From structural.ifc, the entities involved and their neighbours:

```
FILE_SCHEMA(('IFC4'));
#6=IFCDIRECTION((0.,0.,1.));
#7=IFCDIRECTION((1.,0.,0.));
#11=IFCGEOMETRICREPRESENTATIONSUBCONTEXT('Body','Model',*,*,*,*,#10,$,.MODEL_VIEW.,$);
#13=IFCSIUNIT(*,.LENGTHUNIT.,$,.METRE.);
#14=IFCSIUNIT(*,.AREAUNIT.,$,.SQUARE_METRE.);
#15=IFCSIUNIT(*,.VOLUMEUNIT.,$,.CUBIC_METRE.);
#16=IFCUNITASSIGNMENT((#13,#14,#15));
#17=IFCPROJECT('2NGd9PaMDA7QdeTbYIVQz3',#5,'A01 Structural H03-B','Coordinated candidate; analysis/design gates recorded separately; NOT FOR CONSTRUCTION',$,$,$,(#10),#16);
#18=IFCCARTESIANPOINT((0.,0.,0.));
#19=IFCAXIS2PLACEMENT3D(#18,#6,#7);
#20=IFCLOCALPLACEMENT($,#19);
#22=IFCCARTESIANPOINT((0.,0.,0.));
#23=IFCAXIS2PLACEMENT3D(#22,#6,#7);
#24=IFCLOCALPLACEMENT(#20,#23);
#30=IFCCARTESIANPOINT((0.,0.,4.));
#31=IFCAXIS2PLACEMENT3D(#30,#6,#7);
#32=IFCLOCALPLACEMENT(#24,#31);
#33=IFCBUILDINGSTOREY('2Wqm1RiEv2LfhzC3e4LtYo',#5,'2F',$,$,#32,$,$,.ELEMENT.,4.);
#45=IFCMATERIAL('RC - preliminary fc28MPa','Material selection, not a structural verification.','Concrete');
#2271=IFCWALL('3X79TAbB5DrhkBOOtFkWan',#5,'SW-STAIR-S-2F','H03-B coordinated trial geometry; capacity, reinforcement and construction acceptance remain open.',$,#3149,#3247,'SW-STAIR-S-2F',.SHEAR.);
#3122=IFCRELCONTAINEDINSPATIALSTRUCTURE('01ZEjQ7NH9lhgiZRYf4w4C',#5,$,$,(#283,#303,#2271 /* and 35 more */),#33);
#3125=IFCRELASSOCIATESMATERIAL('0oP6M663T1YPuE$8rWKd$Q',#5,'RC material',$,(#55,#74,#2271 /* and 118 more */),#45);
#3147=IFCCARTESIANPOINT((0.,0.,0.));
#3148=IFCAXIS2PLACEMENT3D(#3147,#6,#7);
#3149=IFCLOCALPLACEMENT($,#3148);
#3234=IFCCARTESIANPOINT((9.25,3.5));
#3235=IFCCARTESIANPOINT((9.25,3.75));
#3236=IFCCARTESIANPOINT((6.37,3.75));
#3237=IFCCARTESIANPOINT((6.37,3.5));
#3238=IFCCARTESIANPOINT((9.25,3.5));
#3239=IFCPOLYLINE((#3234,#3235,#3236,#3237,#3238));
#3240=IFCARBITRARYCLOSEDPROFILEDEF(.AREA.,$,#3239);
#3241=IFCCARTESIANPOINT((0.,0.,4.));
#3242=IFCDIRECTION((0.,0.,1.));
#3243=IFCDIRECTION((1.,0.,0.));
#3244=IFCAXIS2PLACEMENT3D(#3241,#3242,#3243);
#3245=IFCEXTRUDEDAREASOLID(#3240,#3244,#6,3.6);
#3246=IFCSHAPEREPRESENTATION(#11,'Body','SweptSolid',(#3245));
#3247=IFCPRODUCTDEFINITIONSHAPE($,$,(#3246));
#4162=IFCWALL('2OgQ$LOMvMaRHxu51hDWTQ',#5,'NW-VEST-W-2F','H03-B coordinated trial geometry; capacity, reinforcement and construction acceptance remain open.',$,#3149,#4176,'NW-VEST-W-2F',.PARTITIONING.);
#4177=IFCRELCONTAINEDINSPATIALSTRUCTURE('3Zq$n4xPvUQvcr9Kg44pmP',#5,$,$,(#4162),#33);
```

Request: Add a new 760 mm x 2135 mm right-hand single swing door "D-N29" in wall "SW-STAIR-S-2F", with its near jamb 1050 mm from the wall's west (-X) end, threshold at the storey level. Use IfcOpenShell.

```python
import numpy as np
import ifcopenshell
import ifcopenshell.api.feature
import ifcopenshell.api.geometry
import ifcopenshell.api.root
import ifcopenshell.api.spatial
import ifcopenshell.geom
import ifcopenshell.util.element
import ifcopenshell.util.placement
import ifcopenshell.util.representation
import ifcopenshell.util.shape
import ifcopenshell.util.unit

model = ifcopenshell.open("structural.ifc")
unit_scale = ifcopenshell.util.unit.calculate_unit_scale(model)
settings = ifcopenshell.geom.settings()


def volume(element):
    """Net volume in cubic metres, openings subtracted."""
    shape = ifcopenshell.geom.create_shape(settings, element)
    return ifcopenshell.util.shape.get_volume(shape.geometry)


wall = model.by_guid("3X79TAbB5DrhkBOOtFkWan")
storey = ifcopenshell.util.element.get_container(wall, ifc_class="IfcBuildingStorey")
context = ifcopenshell.util.representation.get_context(model, "Model", "Body", "MODEL_VIEW")
before = volume(wall)

width, height, from_end, sill = 0.76, 2.135, 1.05, 0.0  # metres

# The wall runs along its own X axis, and the end named is its -X end.
wall_shape = ifcopenshell.geom.create_shape(settings, wall)
x, y, z = ifcopenshell.util.shape.get_vertices(wall_shape.geometry).T
start = x.min() + from_end
face, thickness = float(y.min()), float(y.max() - y.min())
wall_matrix = ifcopenshell.util.placement.get_local_placement(wall.ObjectPlacement)
level = ifcopenshell.util.placement.get_local_placement(storey.ObjectPlacement)[2, 3]


def in_wall(x, y):
    """Placement at x, y metres in the wall's axes, at sill height."""
    matrix = wall_matrix.copy()
    matrix[:, 3] = wall_matrix @ np.array([x / unit_scale, y / unit_scale, 0.0, 1.0])
    matrix[2, 3] = level + sill / unit_scale
    return matrix


# Opening: a box that overshoots both wall faces by 50 mm.
opening = ifcopenshell.api.root.create_entity(model, ifc_class="IfcOpeningElement", predefined_type="OPENING")
box = ifcopenshell.api.geometry.add_wall_representation(
    model, context=context, length=width, height=height, thickness=thickness + 0.1
)
ifcopenshell.api.geometry.assign_representation(model, product=opening, representation=box)
ifcopenshell.api.geometry.edit_object_placement(model, product=opening, matrix=in_wall(start, face - 0.05), is_si=False)
ifcopenshell.api.feature.add_feature(model, feature=opening, element=wall)

door = ifcopenshell.api.root.create_entity(model, ifc_class="IfcDoor", name="D-N29", predefined_type="DOOR")
door.OverallWidth, door.OverallHeight = width / unit_scale, height / unit_scale
door.OperationType = "SINGLE_SWING_RIGHT"
body = ifcopenshell.api.geometry.add_door_representation(
    model,
    context=context,
    overall_width=door.OverallWidth,
    overall_height=door.OverallHeight,
    operation_type="SINGLE_SWING_RIGHT",
    lining_properties={"LiningDepth": thickness / unit_scale, "ThresholdDepth": thickness / unit_scale},
)
ifcopenshell.api.geometry.assign_representation(model, product=door, representation=body)
ifcopenshell.api.spatial.assign_container(model, products=[door], relating_structure=storey)
ifcopenshell.api.feature.add_filling(model, opening=opening, element=door)

# The lining spans the wall, so the door starts at the wall face.
ifcopenshell.api.geometry.edit_object_placement(model, product=door, matrix=in_wall(start, face), is_si=False)

after = volume(wall)

print(f"wall volume {before:.3f} -> {after:.3f} m3")

model.write("structural_v2.ifc")
```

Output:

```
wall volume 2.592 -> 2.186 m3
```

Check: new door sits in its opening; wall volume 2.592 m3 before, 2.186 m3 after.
